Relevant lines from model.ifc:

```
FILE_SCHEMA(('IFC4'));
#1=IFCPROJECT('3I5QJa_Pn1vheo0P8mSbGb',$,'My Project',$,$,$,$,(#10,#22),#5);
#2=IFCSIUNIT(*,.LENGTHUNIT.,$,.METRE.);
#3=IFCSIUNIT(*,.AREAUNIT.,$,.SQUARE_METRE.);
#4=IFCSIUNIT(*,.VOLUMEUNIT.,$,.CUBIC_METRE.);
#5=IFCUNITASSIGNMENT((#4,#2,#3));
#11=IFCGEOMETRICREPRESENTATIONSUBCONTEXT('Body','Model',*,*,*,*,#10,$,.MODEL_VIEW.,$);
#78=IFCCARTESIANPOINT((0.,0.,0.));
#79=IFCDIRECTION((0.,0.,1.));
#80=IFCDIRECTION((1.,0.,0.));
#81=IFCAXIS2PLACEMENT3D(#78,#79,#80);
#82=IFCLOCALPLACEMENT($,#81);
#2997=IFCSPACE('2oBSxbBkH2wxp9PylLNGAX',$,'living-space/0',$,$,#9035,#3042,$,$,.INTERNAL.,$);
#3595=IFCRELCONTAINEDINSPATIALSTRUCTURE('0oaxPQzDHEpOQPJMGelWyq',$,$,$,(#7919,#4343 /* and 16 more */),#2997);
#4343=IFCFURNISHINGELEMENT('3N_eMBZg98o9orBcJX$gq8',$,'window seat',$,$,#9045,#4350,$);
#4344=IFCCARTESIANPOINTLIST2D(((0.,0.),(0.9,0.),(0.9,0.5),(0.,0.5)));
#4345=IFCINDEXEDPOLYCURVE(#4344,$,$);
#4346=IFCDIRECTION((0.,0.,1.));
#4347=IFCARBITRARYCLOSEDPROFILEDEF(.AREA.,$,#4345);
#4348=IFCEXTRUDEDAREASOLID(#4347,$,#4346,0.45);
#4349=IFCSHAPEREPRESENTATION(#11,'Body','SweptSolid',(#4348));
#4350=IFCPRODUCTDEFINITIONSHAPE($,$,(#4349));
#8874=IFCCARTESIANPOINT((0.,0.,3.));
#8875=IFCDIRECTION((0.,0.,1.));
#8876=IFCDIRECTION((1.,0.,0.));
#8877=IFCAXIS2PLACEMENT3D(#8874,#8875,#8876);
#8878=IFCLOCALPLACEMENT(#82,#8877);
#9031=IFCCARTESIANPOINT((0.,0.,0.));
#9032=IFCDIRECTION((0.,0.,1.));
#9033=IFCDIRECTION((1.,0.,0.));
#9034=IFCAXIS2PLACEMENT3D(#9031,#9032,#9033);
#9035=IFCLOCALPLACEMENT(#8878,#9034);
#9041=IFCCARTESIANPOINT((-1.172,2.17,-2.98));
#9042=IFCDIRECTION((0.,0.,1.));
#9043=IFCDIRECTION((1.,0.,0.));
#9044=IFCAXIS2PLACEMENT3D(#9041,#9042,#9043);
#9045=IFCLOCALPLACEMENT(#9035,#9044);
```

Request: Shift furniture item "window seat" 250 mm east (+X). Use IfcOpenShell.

```python
import ifcopenshell
import ifcopenshell.api.geometry
import ifcopenshell.util.placement
import ifcopenshell.util.unit

model = ifcopenshell.open("model.ifc")
unit_scale = ifcopenshell.util.unit.calculate_unit_scale(model)

item = model.by_id(4343)
matrix = ifcopenshell.util.placement.get_local_placement(item.ObjectPlacement)
matrix[0, 3] += 0.25 / unit_scale
ifcopenshell.api.geometry.edit_object_placement(model, product=item, matrix=matrix, is_si=False)

print(ifcopenshell.util.placement.get_local_placement(item.ObjectPlacement).round(3) + 0.0)

model.write("model_updated.ifc")
```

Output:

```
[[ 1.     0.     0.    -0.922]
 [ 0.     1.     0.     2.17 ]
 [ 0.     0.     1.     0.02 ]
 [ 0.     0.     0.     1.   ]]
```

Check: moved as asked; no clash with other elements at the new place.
